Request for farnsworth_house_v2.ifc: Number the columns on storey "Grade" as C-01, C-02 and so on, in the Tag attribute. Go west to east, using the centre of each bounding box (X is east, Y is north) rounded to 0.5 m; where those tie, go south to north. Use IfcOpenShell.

First a look at what the model holds.

```python
import ifcopenshell
import ifcopenshell.util.element
import ifcopenshell.util.placement

model = ifcopenshell.open("farnsworth_house_v2.ifc")
print(model.schema)
storey = next(s for s in model.by_type("IfcBuildingStorey") if s.Name == "Grade")
columns = [e for e in ifcopenshell.util.element.get_decomposition(storey) if e.is_a("IfcColumn")]
for e in sorted(columns, key=lambda e: e.id()):
    origin = ifcopenshell.util.placement.get_local_placement(e.ObjectPlacement)[:3, 3]
    print(e.id(), e.Tag, e.Name, origin.round(2) + 0.0, sep=" | ")
```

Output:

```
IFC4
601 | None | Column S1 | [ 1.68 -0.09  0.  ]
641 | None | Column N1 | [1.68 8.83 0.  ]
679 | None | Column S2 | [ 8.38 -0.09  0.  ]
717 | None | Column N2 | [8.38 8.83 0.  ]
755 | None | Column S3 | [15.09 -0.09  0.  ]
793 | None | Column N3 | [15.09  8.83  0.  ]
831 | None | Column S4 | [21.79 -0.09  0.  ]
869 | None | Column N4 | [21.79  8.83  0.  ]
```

```python
import ifcopenshell
import ifcopenshell.geom
import ifcopenshell.util.element
import ifcopenshell.util.shape

model = ifcopenshell.open("farnsworth_house_v2.ifc")
settings = ifcopenshell.geom.settings()
settings.set("use-world-coords", True)


def centre(element):
    shape = ifcopenshell.geom.create_shape(settings, element)
    return ifcopenshell.util.shape.get_bbox_centroid(shape.geometry)


storey = next(s for s in model.by_type("IfcBuildingStorey") if s.Name == "Grade")
columns = [e for e in ifcopenshell.util.element.get_decomposition(storey) if e.is_a("IfcColumn")]

# Insertion points can sit at a corner or the storey origin, so sort by the geometry (in metres).
centres = {e: centre(e) for e in columns}
columns.sort(key=lambda e: (round(centres[e][0] / 0.5), centres[e][1]))

for i, e in enumerate(columns, start=1):
    number = f"C-{i:02d}"
    e.Tag = number
    print(e.id(), number)

model.write("farnsworth_house_v2_v2.ifc")
```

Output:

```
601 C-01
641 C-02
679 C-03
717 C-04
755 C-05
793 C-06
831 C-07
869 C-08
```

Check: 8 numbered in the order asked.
